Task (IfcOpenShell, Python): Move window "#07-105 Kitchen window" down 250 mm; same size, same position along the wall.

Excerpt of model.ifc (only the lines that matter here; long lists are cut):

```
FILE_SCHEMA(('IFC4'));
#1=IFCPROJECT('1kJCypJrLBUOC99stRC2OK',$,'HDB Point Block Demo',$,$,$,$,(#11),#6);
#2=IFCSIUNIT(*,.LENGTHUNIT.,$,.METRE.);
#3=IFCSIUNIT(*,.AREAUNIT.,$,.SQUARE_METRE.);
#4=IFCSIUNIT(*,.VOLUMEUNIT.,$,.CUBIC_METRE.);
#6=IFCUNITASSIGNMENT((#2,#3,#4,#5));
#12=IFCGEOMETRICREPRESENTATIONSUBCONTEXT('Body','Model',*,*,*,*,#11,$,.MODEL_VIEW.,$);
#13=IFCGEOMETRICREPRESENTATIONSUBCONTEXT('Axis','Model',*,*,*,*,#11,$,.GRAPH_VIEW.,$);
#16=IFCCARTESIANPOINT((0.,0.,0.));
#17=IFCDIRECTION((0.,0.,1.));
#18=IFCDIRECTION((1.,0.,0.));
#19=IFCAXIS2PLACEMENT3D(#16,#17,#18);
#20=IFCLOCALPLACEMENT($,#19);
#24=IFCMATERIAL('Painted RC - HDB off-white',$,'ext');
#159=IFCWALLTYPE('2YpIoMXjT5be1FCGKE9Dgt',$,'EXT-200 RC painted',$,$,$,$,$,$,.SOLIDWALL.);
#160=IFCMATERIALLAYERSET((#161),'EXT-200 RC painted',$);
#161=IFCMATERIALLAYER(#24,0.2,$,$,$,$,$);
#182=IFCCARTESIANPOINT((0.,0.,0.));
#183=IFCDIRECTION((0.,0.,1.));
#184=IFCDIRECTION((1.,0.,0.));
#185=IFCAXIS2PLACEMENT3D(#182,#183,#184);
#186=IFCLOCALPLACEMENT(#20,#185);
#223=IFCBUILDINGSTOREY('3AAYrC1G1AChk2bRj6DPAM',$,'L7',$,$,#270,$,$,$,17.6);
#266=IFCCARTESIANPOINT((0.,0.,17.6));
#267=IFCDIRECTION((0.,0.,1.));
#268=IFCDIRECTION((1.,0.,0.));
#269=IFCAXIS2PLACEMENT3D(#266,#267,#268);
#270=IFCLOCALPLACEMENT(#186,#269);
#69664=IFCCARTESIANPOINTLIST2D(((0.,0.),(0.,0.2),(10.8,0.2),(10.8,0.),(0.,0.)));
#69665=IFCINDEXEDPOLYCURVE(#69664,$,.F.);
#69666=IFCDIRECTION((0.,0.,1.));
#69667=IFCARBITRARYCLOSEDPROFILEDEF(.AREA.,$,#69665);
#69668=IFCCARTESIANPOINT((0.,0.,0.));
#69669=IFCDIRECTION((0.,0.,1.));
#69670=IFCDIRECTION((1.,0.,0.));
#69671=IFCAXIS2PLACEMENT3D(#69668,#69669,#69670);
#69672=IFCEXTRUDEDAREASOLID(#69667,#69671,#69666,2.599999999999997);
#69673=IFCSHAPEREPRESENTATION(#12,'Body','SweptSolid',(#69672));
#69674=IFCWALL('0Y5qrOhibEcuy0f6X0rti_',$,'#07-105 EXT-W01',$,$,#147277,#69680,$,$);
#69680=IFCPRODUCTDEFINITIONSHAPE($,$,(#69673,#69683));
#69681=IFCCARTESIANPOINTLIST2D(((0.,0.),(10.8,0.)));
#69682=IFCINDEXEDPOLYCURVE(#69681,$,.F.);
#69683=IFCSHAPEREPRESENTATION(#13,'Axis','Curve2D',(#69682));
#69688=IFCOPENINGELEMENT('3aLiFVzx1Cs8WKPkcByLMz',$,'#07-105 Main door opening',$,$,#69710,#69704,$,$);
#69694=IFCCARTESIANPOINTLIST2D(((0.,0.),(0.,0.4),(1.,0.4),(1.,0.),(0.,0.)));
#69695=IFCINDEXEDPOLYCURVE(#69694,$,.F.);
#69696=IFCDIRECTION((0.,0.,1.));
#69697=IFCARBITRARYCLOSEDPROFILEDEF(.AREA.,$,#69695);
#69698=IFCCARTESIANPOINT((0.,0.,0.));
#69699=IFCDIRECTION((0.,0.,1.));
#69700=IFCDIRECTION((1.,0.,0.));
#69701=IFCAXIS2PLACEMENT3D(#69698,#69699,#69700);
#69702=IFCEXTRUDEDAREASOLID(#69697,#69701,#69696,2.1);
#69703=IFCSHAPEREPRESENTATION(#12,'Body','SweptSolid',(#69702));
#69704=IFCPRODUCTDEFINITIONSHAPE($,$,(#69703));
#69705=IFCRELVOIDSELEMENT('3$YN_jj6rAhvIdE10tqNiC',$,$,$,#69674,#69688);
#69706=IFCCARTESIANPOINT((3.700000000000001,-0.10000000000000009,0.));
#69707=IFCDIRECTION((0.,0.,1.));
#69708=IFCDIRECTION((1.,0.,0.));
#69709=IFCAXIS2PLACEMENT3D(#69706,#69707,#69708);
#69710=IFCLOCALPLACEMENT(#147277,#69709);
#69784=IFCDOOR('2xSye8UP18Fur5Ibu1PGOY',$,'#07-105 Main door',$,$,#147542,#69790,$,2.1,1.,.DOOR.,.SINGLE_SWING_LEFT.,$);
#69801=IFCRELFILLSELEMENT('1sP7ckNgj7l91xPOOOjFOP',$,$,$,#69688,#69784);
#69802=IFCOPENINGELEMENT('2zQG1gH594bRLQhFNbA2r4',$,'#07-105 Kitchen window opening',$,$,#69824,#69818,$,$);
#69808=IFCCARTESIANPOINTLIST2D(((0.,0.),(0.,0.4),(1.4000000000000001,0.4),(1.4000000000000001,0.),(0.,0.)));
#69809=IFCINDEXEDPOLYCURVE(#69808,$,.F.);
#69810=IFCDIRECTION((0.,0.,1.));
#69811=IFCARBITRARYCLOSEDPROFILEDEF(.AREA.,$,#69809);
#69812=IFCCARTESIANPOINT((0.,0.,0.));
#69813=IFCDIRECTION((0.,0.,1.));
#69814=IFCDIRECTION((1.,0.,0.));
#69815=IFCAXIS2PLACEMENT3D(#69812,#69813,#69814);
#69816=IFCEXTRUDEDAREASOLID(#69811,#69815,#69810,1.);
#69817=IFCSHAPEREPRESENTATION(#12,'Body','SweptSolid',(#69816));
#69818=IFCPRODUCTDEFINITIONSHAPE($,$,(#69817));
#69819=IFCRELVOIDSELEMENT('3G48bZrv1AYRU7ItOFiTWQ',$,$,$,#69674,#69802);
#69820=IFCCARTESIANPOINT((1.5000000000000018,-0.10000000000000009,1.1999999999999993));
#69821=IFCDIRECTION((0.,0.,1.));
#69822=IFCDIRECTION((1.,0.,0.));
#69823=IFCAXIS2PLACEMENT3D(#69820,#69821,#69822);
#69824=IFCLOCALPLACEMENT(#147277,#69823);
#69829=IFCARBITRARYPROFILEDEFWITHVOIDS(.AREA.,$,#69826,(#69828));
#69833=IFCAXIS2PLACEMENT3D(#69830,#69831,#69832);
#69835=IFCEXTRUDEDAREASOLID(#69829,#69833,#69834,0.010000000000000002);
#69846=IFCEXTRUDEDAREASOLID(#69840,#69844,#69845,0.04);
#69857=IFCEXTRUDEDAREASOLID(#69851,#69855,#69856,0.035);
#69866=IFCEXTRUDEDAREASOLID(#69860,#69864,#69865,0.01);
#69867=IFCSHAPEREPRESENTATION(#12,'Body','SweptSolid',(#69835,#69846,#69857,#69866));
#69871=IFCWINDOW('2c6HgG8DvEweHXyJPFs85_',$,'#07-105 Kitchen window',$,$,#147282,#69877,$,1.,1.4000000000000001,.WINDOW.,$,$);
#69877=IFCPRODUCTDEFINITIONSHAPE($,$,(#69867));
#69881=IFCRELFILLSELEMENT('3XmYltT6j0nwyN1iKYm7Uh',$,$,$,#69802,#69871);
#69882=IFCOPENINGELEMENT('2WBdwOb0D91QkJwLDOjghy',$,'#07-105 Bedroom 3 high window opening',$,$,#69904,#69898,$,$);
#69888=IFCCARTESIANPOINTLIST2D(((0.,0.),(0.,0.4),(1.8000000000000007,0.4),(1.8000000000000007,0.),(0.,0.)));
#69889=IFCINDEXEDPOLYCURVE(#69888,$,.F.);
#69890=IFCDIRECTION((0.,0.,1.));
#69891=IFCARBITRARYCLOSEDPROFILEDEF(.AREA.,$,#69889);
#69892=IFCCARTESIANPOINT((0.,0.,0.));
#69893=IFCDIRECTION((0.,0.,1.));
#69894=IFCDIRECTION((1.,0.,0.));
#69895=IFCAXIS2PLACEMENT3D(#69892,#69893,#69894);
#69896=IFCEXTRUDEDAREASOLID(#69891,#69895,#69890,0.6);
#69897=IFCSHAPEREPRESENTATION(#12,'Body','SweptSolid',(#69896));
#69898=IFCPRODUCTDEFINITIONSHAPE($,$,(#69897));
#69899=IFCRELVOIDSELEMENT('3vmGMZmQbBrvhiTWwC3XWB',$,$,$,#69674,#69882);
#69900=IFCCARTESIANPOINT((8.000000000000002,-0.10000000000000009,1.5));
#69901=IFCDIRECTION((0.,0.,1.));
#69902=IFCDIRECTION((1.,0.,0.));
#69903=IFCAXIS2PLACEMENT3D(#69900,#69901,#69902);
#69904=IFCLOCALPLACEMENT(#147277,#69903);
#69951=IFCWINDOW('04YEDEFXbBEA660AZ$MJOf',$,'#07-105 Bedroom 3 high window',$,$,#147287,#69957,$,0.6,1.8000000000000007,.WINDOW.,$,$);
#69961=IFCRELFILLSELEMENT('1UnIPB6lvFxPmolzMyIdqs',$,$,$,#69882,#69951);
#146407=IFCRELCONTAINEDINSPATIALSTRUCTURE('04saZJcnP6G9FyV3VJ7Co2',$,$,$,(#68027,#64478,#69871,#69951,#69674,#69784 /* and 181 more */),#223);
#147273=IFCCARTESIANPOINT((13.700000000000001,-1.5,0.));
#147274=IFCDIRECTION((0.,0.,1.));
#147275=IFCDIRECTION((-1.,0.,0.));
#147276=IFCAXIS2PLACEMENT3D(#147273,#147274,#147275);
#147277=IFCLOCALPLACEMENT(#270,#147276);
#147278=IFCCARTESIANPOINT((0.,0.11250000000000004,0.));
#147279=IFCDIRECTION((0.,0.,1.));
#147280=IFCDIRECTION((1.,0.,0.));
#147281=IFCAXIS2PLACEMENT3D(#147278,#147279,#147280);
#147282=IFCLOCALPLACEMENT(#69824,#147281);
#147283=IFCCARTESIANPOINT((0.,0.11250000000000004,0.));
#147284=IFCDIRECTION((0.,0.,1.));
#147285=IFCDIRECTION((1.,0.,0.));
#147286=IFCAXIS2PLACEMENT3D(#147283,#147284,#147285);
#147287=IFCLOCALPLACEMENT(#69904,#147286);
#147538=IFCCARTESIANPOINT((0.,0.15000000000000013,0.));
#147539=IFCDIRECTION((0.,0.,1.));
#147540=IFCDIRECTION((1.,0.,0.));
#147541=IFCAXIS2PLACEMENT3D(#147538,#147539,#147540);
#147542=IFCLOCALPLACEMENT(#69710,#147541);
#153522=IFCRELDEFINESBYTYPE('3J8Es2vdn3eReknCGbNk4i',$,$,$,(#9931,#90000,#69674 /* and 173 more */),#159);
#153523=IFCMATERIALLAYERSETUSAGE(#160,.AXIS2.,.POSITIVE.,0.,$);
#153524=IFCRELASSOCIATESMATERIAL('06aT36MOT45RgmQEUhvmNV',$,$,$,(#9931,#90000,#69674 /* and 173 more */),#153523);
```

```python
import numpy as np
import ifcopenshell
import ifcopenshell.api.geometry
import ifcopenshell.util.placement
import ifcopenshell.util.unit

model = ifcopenshell.open("model.ifc")
unit_scale = ifcopenshell.util.unit.calculate_unit_scale(model)

window = model.by_guid("2c6HgG8DvEweHXyJPFs85_")
opening = window.FillsVoids[0].RelatingOpeningElement
dz = -0.25

shift = np.array([0.0, 0.0, dz])
# The window is placed relative to its opening, so it follows when the opening moves.
matrix = ifcopenshell.util.placement.get_local_placement(opening.ObjectPlacement)
matrix[:3, 3] += shift
ifcopenshell.api.geometry.edit_object_placement(
    model, product=opening, matrix=matrix, is_si=False, should_transform_children=True
)

print(f"moved by {dz * unit_scale:+.3f} m")

model.write("model_rev.ifc")
```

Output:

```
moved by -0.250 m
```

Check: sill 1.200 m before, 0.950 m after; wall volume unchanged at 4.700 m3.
